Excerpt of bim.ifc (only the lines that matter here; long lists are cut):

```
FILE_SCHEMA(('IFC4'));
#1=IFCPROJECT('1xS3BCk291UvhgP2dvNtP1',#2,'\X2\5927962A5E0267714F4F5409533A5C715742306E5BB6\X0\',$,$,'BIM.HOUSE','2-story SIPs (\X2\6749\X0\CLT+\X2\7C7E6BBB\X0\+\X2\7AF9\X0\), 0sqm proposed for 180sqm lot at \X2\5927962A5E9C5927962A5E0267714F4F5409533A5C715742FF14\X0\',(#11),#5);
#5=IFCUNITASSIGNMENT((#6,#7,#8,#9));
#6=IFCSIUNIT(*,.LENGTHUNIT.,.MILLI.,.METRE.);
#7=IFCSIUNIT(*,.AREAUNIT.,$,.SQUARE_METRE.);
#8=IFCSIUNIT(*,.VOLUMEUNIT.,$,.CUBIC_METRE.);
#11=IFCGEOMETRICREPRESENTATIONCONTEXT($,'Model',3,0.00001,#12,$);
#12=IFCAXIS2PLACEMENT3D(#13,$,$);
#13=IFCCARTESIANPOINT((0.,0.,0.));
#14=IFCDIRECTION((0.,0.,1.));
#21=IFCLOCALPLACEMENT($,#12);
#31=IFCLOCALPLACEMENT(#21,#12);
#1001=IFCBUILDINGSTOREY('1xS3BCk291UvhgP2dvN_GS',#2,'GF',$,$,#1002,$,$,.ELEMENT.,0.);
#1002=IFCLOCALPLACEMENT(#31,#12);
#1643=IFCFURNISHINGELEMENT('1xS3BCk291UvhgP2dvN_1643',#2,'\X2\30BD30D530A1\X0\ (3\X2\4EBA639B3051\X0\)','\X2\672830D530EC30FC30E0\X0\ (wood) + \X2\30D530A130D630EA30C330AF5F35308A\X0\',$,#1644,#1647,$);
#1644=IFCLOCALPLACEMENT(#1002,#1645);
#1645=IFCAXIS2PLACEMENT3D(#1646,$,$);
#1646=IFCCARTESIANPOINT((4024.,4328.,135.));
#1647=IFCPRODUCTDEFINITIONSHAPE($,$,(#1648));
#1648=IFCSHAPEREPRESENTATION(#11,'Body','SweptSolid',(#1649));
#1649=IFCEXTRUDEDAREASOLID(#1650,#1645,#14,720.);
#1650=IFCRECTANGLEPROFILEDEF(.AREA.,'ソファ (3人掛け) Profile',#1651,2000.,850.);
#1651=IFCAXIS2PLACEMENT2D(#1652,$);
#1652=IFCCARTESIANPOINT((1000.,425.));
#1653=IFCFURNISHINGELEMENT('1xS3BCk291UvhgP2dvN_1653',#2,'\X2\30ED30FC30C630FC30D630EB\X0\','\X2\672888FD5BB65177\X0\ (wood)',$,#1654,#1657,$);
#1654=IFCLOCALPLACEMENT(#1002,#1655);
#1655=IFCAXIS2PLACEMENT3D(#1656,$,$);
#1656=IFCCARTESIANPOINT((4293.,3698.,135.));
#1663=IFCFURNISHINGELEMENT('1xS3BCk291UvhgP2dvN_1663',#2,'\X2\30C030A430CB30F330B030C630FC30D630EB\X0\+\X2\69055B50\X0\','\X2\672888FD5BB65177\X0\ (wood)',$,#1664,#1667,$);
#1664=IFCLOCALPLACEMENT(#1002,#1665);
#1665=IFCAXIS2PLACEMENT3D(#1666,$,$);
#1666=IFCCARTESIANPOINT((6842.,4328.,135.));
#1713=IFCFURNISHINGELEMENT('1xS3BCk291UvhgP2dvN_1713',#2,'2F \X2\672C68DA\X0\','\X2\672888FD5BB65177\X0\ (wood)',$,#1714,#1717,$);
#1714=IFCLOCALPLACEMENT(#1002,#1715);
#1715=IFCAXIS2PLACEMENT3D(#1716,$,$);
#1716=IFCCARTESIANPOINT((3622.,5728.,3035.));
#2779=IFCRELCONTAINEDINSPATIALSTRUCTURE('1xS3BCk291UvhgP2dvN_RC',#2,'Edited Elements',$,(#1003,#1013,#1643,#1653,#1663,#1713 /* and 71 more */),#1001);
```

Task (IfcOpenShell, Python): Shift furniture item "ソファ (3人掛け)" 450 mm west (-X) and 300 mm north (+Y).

```python
import ifcopenshell
import ifcopenshell.api.geometry
import ifcopenshell.util.placement
import ifcopenshell.util.unit

model = ifcopenshell.open("bim.ifc")
unit_scale = ifcopenshell.util.unit.calculate_unit_scale(model)

item = model.by_id(1643)
matrix = ifcopenshell.util.placement.get_local_placement(item.ObjectPlacement)
matrix[0, 3] -= 0.45 / unit_scale
matrix[1, 3] += 0.3 / unit_scale
ifcopenshell.api.geometry.edit_object_placement(model, product=item, matrix=matrix, is_si=False)

print(ifcopenshell.util.placement.get_local_placement(item.ObjectPlacement).round(3) + 0.0)

model.write("bim_updated.ifc")
```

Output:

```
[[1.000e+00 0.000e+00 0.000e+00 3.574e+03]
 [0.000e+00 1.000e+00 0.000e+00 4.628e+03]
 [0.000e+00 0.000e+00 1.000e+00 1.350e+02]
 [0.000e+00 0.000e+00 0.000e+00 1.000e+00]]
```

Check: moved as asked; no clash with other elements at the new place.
